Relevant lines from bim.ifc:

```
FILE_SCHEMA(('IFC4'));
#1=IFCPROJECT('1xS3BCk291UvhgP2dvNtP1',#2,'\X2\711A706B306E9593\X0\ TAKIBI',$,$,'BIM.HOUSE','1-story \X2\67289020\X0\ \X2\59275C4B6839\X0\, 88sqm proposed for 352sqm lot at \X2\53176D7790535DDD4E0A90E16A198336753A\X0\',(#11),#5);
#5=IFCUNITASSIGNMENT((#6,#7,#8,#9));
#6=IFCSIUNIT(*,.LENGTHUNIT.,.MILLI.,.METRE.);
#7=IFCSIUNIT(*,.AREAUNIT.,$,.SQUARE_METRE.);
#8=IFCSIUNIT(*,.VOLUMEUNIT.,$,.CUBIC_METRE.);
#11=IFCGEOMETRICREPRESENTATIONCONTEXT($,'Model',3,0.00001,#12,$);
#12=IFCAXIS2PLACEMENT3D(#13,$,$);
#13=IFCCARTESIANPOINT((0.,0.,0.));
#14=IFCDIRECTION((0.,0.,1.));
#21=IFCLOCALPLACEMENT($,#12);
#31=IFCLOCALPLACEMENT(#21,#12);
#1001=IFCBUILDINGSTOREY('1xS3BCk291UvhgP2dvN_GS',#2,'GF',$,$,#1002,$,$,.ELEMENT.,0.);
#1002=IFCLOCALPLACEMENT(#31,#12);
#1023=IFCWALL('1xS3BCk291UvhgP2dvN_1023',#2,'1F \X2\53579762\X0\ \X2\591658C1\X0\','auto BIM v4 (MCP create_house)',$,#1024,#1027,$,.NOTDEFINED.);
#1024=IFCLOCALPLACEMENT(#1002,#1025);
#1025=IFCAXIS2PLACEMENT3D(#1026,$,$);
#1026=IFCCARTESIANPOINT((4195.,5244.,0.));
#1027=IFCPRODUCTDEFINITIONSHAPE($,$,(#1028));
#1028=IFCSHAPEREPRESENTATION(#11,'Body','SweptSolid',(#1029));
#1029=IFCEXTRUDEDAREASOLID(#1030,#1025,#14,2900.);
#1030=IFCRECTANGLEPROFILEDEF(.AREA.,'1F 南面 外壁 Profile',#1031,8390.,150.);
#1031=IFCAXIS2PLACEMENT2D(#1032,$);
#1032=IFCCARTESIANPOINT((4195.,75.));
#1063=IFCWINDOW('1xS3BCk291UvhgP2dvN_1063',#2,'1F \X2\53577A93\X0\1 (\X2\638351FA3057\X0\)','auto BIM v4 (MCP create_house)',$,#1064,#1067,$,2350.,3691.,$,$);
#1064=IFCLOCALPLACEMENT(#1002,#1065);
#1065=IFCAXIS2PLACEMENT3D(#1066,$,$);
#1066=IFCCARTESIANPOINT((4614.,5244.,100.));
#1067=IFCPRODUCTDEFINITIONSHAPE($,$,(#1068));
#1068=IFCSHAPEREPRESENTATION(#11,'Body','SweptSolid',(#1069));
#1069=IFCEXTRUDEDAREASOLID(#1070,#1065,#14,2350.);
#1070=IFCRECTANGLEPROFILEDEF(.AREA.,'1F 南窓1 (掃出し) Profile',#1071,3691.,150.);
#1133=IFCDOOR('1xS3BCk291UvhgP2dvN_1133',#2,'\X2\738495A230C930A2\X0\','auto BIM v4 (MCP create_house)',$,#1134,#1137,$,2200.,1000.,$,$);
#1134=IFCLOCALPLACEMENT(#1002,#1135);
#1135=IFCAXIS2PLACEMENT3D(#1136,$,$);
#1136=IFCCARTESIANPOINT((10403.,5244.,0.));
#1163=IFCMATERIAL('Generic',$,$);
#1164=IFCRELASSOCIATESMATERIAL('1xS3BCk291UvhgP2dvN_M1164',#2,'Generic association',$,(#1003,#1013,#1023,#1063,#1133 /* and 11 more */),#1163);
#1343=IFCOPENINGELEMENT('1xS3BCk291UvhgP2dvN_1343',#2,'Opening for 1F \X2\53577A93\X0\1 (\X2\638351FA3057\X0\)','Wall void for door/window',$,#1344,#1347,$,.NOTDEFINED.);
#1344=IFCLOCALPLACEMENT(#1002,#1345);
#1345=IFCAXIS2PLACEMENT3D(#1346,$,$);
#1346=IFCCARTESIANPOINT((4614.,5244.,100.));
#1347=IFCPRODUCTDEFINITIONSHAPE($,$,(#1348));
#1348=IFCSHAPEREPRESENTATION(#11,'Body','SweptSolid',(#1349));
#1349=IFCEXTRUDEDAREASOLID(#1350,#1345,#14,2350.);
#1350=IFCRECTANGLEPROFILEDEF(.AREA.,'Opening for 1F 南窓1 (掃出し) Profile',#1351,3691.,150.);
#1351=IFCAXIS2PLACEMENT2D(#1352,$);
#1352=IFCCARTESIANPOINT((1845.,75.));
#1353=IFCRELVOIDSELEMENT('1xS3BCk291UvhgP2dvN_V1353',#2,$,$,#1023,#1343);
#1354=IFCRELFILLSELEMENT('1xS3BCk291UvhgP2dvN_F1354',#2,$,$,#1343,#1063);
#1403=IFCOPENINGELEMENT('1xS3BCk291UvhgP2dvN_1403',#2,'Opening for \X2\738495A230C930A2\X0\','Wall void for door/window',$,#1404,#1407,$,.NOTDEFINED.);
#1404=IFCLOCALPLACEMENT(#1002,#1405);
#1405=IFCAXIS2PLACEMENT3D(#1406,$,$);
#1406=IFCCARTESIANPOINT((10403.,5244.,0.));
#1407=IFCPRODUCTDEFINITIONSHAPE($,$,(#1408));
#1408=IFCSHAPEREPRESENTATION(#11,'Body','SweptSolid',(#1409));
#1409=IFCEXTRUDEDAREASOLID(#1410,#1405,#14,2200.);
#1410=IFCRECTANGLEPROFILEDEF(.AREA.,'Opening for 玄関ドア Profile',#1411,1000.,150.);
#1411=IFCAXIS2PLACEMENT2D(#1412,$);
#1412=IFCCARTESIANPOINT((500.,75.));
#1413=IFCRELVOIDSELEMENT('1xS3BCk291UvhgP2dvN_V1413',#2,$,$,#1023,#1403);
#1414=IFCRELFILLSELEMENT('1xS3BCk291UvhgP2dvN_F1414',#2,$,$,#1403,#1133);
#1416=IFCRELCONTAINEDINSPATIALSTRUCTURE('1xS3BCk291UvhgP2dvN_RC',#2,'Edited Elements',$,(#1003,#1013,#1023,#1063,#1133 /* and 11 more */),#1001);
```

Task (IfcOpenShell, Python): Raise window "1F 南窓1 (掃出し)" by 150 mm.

```python
import numpy as np
import ifcopenshell
import ifcopenshell.api.geometry
import ifcopenshell.util.placement
import ifcopenshell.util.unit

model = ifcopenshell.open("bim.ifc")
unit_scale = ifcopenshell.util.unit.calculate_unit_scale(model)

window = model.by_guid("1xS3BCk291UvhgP2dvN_1063")
opening = window.FillsVoids[0].RelatingOpeningElement
dz = 0.15 / unit_scale

shift = np.array([0.0, 0.0, dz])
# The window is not placed relative to its opening, so move both.
for product in (opening, window):
    matrix = ifcopenshell.util.placement.get_local_placement(product.ObjectPlacement)
    matrix[:3, 3] += shift
    ifcopenshell.api.geometry.edit_object_placement(model, product=product, matrix=matrix, is_si=False)

print(f"moved by {dz * unit_scale:+.3f} m")

model.write("bim_updated.ifc")
```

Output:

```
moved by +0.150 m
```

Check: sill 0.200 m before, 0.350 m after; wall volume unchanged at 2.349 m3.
